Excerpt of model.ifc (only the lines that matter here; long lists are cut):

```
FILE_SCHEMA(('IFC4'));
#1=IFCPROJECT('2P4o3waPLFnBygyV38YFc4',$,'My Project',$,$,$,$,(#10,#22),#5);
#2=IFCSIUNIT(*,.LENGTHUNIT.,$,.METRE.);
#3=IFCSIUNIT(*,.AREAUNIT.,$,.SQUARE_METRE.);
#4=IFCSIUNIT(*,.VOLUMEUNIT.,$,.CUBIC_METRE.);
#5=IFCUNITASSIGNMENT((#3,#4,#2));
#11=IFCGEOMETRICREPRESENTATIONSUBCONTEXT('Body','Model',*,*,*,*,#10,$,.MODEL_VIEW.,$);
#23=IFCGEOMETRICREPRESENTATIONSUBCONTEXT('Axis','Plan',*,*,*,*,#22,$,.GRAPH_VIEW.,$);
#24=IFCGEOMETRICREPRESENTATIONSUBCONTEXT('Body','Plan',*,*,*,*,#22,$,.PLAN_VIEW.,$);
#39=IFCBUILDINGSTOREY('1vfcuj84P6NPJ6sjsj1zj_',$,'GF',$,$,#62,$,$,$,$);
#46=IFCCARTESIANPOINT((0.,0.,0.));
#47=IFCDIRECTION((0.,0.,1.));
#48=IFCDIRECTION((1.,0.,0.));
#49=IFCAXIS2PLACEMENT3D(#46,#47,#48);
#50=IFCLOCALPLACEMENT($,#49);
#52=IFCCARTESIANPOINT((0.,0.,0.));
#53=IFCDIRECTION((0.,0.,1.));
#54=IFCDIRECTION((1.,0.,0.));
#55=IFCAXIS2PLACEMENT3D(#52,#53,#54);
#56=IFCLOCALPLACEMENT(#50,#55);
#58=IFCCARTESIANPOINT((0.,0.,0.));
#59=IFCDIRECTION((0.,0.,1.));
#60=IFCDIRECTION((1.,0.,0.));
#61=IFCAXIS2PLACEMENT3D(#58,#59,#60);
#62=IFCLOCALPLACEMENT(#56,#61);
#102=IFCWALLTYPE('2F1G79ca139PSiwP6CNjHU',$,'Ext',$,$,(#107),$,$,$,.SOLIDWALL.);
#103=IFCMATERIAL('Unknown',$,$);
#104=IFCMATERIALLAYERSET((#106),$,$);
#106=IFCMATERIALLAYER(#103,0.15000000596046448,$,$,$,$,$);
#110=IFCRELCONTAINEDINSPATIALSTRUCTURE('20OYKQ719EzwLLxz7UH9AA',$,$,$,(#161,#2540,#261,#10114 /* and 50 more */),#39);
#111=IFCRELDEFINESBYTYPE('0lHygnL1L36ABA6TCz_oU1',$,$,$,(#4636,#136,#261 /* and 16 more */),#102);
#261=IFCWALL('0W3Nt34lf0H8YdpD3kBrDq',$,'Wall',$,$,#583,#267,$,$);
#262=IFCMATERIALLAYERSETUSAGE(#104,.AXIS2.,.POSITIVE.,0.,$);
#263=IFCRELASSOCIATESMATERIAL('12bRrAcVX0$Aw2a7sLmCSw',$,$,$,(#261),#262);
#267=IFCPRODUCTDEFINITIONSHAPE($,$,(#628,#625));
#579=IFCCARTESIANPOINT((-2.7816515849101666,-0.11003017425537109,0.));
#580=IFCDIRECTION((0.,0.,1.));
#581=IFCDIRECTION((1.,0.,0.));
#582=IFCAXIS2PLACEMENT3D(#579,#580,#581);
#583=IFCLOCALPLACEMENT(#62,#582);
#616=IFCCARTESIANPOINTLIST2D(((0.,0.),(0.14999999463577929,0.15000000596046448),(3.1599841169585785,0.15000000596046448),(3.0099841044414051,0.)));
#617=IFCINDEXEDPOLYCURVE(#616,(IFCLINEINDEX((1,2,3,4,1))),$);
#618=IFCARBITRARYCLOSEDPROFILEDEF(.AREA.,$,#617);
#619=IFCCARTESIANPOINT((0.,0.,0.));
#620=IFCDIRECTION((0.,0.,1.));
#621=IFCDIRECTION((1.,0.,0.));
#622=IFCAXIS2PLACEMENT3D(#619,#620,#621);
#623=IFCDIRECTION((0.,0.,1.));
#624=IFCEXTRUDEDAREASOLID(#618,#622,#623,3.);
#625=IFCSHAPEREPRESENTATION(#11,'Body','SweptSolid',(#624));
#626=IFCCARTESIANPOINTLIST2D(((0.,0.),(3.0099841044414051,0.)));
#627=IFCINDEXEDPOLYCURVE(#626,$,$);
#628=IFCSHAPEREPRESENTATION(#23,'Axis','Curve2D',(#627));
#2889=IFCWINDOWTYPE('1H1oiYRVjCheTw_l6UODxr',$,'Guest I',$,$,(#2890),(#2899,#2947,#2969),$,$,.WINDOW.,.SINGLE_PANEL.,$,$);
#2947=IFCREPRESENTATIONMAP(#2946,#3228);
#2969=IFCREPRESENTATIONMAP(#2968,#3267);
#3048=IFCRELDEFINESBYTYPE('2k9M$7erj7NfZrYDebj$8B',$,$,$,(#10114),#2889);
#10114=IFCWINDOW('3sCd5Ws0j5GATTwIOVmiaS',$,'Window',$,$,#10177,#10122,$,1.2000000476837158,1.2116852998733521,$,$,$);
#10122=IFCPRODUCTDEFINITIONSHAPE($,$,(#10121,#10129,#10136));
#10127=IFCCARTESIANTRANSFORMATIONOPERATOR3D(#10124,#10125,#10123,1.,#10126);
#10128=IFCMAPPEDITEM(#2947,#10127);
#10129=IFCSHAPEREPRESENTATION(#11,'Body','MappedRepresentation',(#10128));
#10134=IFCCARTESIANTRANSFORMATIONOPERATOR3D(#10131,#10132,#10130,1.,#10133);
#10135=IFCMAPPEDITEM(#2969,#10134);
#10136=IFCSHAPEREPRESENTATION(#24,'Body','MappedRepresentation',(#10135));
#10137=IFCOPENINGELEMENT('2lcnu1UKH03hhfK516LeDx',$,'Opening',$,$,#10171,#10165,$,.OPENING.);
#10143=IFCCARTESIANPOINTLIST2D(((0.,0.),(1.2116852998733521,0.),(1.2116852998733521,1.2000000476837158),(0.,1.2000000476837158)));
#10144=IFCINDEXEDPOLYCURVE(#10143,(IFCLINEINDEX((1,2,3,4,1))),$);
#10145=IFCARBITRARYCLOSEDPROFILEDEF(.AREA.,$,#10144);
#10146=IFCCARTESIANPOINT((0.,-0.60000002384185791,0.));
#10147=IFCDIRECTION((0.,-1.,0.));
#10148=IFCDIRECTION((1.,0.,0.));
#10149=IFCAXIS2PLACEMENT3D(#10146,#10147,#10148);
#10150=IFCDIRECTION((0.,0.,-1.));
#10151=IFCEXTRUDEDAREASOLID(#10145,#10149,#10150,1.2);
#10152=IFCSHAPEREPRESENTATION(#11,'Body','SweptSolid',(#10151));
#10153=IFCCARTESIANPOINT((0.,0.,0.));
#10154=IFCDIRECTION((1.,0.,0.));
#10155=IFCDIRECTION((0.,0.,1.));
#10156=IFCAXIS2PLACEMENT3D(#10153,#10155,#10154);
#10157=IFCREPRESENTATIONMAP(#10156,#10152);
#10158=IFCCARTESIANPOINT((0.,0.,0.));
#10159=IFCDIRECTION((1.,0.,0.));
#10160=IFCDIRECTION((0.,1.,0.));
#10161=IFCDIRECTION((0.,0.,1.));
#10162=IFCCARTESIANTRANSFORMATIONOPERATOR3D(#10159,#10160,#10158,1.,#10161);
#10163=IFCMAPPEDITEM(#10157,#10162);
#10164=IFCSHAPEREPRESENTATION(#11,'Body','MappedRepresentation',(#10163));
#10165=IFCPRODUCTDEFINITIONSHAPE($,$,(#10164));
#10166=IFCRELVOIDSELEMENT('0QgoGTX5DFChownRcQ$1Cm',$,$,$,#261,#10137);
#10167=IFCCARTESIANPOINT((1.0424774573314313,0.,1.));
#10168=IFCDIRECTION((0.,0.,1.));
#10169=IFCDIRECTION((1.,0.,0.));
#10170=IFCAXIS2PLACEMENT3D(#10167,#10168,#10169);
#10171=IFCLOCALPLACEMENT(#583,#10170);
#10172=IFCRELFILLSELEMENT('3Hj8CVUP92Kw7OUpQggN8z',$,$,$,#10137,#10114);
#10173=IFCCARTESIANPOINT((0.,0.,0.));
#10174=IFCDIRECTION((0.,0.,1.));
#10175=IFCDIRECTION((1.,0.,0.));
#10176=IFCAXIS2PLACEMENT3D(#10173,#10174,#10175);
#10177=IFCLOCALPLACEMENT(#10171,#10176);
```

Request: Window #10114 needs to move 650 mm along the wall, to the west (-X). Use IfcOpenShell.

```python
import ifcopenshell
import ifcopenshell.api.geometry
import ifcopenshell.util.placement

model = ifcopenshell.open("model.ifc")

window = model.by_guid("3sCd5Ws0j5GATTwIOVmiaS")
opening = window.FillsVoids[0].RelatingOpeningElement
wall = opening.VoidsElements[0].RelatingBuildingElement

wall_matrix = ifcopenshell.util.placement.get_local_placement(wall.ObjectPlacement)
shift = wall_matrix[:3, 0] * -0.65
before = ifcopenshell.util.placement.get_local_placement(window.ObjectPlacement)[:3, 3].copy()

# The window is placed relative to its opening, so it follows when the opening moves.
matrix = ifcopenshell.util.placement.get_local_placement(opening.ObjectPlacement)
matrix[:3, 3] += shift
ifcopenshell.api.geometry.edit_object_placement(
    model, product=opening, matrix=matrix, is_si=False, should_transform_children=True
)

after = ifcopenshell.util.placement.get_local_placement(window.ObjectPlacement)[:3, 3]
print("window moved by", (after - before).round(3) + 0.0)

model.write("model_updated.ifc")
```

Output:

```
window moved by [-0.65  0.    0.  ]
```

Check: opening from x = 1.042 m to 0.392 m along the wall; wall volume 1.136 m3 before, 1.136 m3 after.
